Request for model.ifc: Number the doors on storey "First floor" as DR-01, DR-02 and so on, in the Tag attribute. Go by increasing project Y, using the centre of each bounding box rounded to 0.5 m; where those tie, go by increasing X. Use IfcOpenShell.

First a look at what the model holds.

```python
import ifcopenshell
import ifcopenshell.util.element
import ifcopenshell.util.placement

model = ifcopenshell.open("model.ifc")
print(model.schema)
storey = next(s for s in model.by_type("IfcBuildingStorey") if s.Name == "First floor")
doors = [e for e in ifcopenshell.util.element.get_decomposition(storey) if e.is_a("IfcDoor")]
for e in sorted(doors, key=lambda e: e.id()):
    origin = ifcopenshell.util.placement.get_local_placement(e.ObjectPlacement)[:3, 3]
    print(e.id(), e.Tag, e.Name, origin.round(2) + 0.0, sep=" | ")
```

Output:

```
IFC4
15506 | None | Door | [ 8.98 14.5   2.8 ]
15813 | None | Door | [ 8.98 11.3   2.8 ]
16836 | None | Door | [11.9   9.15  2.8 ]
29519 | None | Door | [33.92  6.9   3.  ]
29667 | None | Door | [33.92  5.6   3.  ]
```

```python
import ifcopenshell
import ifcopenshell.geom
import ifcopenshell.util.element
import ifcopenshell.util.shape

model = ifcopenshell.open("model.ifc")
settings = ifcopenshell.geom.settings()
settings.set("use-world-coords", True)


def centre(element):
    shape = ifcopenshell.geom.create_shape(settings, element)
    return ifcopenshell.util.shape.get_bbox_centroid(shape.geometry)


storey = next(s for s in model.by_type("IfcBuildingStorey") if s.Name == "First floor")
doors = [e for e in ifcopenshell.util.element.get_decomposition(storey) if e.is_a("IfcDoor")]

# Insertion points can sit at a corner or the storey origin, so sort by the geometry (in metres).
centres = {e: centre(e) for e in doors}
doors.sort(key=lambda e: (round(centres[e][1] / 0.5), centres[e][0]))

for i, e in enumerate(doors, start=1):
    number = f"DR-{i:02d}"
    e.Tag = number
    print(e.id(), number)

model.write("model_edited.ifc")
```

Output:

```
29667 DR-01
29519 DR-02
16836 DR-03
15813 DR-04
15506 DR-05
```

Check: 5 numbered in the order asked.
